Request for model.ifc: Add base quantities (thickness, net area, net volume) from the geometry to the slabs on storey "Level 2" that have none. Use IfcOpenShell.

First a look at what the model holds.

```python
import ifcopenshell
import ifcopenshell.util.element
import ifcopenshell.util.unit

model = ifcopenshell.open("model.ifc")
print(model.schema)
for unit_type in ("LENGTHUNIT", "AREAUNIT", "VOLUMEUNIT"):
    print(unit_type, ifcopenshell.util.unit.calculate_unit_scale(model, unit_type))
storey = next(s for s in model.by_type("IfcBuildingStorey") if s.Name == "Level 2")
slabs = [e for e in ifcopenshell.util.element.get_decomposition(storey) if e.is_a("IfcSlab")]
for e in sorted(slabs, key=lambda e: e.id()):
    print(e.id(), e.is_a(), e.Name, list(ifcopenshell.util.element.get_psets(e, qtos_only=True)), sep=" | ")
```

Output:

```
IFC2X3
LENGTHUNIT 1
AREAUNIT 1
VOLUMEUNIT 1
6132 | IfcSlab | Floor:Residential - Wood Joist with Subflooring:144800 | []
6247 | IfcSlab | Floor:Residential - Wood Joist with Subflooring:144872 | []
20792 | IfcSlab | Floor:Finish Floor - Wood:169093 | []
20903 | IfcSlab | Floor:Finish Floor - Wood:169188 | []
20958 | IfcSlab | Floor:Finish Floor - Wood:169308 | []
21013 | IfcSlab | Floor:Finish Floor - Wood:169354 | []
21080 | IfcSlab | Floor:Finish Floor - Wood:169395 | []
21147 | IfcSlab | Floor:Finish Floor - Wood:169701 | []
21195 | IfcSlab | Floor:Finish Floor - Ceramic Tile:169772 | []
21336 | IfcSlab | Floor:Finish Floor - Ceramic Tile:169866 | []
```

```python
import ifcopenshell
import ifcopenshell.api.pset
import ifcopenshell.geom
import ifcopenshell.util.element
import ifcopenshell.util.shape
import ifcopenshell.util.unit

model = ifcopenshell.open("model.ifc")
unit_scale = ifcopenshell.util.unit.calculate_unit_scale(model)
area_scale = ifcopenshell.util.unit.calculate_unit_scale(model, "AREAUNIT")
volume_scale = ifcopenshell.util.unit.calculate_unit_scale(model, "VOLUMEUNIT")
settings = ifcopenshell.geom.settings()

storey = next(s for s in model.by_type("IfcBuildingStorey") if s.Name == "Level 2")
slabs = [e for e in ifcopenshell.util.element.get_decomposition(storey) if e.is_a("IfcSlab")]

for e in sorted(slabs, key=lambda e: e.id()):
    if ifcopenshell.util.element.get_psets(e, qtos_only=True, should_inherit=False):
        continue
    # Geometry comes back in metres, in the element's own axes.
    shape = ifcopenshell.geom.create_shape(settings, e)
    values = {
        "Width": ifcopenshell.util.shape.get_z(shape.geometry) / unit_scale,
        "NetArea": ifcopenshell.util.shape.get_footprint_area(shape.geometry) / area_scale,
        "NetVolume": ifcopenshell.util.shape.get_volume(shape.geometry) / volume_scale,
    }
    qto = ifcopenshell.api.pset.add_qto(model, product=e, name="BaseQuantities")
    ifcopenshell.api.pset.edit_qto(model, qto=qto, properties=values)
    print(e.id(), {k: round(v, 3) for k, v in values.items()})

model.write("model_v2.ifc")
```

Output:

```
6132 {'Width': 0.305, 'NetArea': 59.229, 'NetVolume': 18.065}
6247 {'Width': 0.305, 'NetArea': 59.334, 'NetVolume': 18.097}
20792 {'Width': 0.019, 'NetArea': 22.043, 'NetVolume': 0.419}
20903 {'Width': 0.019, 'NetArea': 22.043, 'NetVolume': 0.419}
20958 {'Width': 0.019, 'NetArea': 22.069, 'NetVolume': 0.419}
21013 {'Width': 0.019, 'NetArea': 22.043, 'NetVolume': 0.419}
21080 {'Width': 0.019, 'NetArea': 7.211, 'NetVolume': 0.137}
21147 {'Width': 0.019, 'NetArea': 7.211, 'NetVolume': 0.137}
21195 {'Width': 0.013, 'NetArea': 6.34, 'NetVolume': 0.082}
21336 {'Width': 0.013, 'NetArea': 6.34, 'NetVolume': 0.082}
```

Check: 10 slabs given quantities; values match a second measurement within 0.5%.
